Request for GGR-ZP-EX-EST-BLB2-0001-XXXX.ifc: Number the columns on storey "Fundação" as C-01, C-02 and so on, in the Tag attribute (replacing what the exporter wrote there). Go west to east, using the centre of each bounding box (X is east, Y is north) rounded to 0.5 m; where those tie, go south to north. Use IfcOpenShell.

First a look at what the model holds.

```python
import ifcopenshell
import ifcopenshell.util.element
import ifcopenshell.util.placement

model = ifcopenshell.open("GGR-ZP-EX-EST-BLB2-0001-XXXX.ifc")
print(model.schema)
storey = next(s for s in model.by_type("IfcBuildingStorey") if s.Name == "Fundação")
columns = [e for e in ifcopenshell.util.element.get_decomposition(storey) if e.is_a("IfcColumn")]
for e in sorted(columns, key=lambda e: e.id()):
    origin = ifcopenshell.util.placement.get_local_placement(e.ObjectPlacement)[:3, 3]
    print(e.id(), e.Tag, e.Name, origin.round(2) + 0.0, sep=" | ")
```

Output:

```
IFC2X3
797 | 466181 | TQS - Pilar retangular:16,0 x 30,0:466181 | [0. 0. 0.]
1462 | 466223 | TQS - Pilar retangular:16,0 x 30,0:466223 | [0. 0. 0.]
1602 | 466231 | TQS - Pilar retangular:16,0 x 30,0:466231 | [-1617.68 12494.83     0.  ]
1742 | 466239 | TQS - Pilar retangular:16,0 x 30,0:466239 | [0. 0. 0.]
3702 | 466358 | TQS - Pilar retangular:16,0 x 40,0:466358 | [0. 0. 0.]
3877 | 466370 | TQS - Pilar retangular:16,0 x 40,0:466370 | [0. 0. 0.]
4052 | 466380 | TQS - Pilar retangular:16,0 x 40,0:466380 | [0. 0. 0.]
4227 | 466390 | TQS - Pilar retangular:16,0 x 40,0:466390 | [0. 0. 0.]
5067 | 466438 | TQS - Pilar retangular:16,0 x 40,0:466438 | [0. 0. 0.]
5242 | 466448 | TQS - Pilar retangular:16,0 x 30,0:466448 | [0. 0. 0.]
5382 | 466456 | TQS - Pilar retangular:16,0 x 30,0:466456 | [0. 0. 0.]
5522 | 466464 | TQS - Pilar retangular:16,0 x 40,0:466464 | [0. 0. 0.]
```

```python
import ifcopenshell
import ifcopenshell.geom
import ifcopenshell.util.element
import ifcopenshell.util.shape

model = ifcopenshell.open("GGR-ZP-EX-EST-BLB2-0001-XXXX.ifc")
settings = ifcopenshell.geom.settings()
settings.set("use-world-coords", True)


def centre(element):
    shape = ifcopenshell.geom.create_shape(settings, element)
    return ifcopenshell.util.shape.get_bbox_centroid(shape.geometry)


storey = next(s for s in model.by_type("IfcBuildingStorey") if s.Name == "Fundação")
columns = [e for e in ifcopenshell.util.element.get_decomposition(storey) if e.is_a("IfcColumn")]

# Insertion points can sit at a corner or the storey origin, so sort by the geometry (in metres).
centres = {e: centre(e) for e in columns}
columns.sort(key=lambda e: (round(centres[e][0] / 0.5), centres[e][1]))

for i, e in enumerate(columns, start=1):
    number = f"C-{i:02d}"
    e.Tag = number
    print(e.id(), number)

model.write("GGR-ZP-EX-EST-BLB2-0001-XXXX_v2.ifc")
```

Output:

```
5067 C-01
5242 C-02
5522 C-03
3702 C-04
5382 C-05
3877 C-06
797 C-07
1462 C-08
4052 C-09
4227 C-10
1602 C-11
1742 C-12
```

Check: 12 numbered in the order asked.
